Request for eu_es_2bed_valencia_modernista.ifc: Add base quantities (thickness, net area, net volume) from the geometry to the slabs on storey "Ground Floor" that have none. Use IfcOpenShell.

First a look at what the model holds.

```python
import ifcopenshell
import ifcopenshell.util.element
import ifcopenshell.util.unit

model = ifcopenshell.open("eu_es_2bed_valencia_modernista.ifc")
print(model.schema)
for unit_type in ("LENGTHUNIT", "AREAUNIT", "VOLUMEUNIT"):
    print(unit_type, ifcopenshell.util.unit.calculate_unit_scale(model, unit_type))
storey = next(s for s in model.by_type("IfcBuildingStorey") if s.Name == "Ground Floor")
slabs = [e for e in ifcopenshell.util.element.get_decomposition(storey) if e.is_a("IfcSlab")]
for e in sorted(slabs, key=lambda e: e.id()):
    print(e.id(), e.is_a(), e.Name, list(ifcopenshell.util.element.get_psets(e, qtos_only=True)), sep=" | ")
```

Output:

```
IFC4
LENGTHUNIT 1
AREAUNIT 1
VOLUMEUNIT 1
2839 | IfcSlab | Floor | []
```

```python
import ifcopenshell
import ifcopenshell.api.pset
import ifcopenshell.geom
import ifcopenshell.util.element
import ifcopenshell.util.shape
import ifcopenshell.util.unit

model = ifcopenshell.open("eu_es_2bed_valencia_modernista.ifc")
unit_scale = ifcopenshell.util.unit.calculate_unit_scale(model)
area_scale = ifcopenshell.util.unit.calculate_unit_scale(model, "AREAUNIT")
volume_scale = ifcopenshell.util.unit.calculate_unit_scale(model, "VOLUMEUNIT")
settings = ifcopenshell.geom.settings()

storey = next(s for s in model.by_type("IfcBuildingStorey") if s.Name == "Ground Floor")
slabs = [e for e in ifcopenshell.util.element.get_decomposition(storey) if e.is_a("IfcSlab")]

for e in sorted(slabs, key=lambda e: e.id()):
    if ifcopenshell.util.element.get_psets(e, qtos_only=True, should_inherit=False):
        continue
    # Geometry comes back in metres, in the element's own axes.
    shape = ifcopenshell.geom.create_shape(settings, e)
    values = {
        "Width": ifcopenshell.util.shape.get_z(shape.geometry) / unit_scale,
        "NetArea": ifcopenshell.util.shape.get_footprint_area(shape.geometry) / area_scale,
        "NetVolume": ifcopenshell.util.shape.get_volume(shape.geometry) / volume_scale,
    }
    qto = ifcopenshell.api.pset.add_qto(model, product=e, name="Qto_SlabBaseQuantities")
    ifcopenshell.api.pset.edit_qto(model, qto=qto, properties=values)
    print(e.id(), {k: round(v, 3) for k, v in values.items()})

model.write("eu_es_2bed_valencia_modernista-out.ifc")
```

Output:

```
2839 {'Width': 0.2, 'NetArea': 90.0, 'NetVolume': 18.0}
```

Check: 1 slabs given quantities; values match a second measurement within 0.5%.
